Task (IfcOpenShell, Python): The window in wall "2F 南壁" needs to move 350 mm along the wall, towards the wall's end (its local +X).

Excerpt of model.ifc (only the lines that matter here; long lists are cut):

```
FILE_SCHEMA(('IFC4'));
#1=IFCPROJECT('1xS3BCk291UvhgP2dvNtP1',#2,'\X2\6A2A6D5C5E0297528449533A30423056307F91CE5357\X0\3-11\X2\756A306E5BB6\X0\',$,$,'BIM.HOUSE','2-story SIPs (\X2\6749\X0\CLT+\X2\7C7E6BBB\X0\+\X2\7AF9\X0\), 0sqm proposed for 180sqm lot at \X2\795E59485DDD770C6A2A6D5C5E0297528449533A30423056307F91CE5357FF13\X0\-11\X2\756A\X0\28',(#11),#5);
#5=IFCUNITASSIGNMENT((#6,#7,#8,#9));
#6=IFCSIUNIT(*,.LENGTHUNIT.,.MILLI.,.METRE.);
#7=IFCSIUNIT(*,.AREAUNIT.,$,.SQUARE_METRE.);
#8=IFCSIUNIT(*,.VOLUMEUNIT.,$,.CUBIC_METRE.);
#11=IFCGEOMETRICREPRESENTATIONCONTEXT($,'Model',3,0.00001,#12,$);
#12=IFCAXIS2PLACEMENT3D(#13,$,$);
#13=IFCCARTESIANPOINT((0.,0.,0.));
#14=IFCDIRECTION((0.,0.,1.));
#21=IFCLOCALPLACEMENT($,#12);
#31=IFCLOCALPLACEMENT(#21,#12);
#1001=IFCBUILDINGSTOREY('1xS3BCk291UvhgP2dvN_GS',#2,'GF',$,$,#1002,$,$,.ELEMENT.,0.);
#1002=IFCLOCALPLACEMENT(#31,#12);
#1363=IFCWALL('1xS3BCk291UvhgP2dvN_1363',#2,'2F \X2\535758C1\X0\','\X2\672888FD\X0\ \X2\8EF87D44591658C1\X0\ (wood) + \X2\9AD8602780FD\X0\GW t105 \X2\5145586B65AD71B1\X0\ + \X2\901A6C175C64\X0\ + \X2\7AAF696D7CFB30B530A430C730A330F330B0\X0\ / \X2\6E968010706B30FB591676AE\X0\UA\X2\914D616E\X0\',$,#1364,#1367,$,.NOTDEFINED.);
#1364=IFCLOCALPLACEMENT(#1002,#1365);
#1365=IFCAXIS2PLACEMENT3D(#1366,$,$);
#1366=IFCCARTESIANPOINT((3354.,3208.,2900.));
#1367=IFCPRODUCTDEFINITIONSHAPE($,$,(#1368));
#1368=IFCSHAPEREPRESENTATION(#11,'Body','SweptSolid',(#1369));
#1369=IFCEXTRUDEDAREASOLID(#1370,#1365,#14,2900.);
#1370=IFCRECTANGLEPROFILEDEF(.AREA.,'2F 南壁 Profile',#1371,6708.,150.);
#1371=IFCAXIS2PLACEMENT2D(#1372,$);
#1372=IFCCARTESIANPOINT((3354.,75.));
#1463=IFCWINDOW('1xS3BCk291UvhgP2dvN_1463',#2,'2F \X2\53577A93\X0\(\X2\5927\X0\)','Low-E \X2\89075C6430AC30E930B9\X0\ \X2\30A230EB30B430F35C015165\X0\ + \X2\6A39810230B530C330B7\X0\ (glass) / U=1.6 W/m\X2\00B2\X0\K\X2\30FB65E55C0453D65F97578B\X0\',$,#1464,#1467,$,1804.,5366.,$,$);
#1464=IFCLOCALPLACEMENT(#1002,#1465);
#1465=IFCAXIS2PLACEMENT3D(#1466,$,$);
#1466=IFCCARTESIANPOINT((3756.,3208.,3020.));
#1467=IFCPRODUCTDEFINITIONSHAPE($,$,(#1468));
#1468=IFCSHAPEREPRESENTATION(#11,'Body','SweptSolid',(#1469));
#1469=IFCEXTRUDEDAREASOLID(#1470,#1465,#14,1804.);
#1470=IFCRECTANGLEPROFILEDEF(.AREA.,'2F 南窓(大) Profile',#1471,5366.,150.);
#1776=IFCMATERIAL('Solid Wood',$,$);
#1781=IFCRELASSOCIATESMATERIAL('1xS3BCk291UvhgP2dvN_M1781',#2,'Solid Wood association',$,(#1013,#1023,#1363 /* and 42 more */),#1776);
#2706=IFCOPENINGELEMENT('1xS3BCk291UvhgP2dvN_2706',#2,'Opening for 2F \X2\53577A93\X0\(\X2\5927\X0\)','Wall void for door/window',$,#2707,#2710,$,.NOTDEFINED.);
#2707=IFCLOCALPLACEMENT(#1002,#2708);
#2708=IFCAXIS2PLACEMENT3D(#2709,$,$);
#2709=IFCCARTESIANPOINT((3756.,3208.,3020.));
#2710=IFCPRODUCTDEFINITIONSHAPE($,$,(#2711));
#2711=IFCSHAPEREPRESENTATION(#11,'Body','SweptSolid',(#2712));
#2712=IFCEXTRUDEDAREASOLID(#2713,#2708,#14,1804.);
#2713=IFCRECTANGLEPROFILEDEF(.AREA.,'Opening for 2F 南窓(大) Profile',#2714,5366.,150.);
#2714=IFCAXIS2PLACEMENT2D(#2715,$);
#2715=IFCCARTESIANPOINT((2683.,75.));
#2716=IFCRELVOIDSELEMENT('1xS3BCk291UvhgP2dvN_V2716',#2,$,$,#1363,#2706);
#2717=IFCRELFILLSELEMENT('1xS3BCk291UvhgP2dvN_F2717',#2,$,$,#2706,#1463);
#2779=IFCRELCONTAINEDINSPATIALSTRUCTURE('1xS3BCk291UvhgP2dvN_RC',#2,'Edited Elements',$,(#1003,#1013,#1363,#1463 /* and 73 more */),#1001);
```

```python
import ifcopenshell
import ifcopenshell.api.geometry
import ifcopenshell.util.placement

model = ifcopenshell.open("model.ifc")

window = model.by_guid("1xS3BCk291UvhgP2dvN_1463")
opening = window.FillsVoids[0].RelatingOpeningElement
wall = opening.VoidsElements[0].RelatingBuildingElement

wall_matrix = ifcopenshell.util.placement.get_local_placement(wall.ObjectPlacement)
shift = wall_matrix[:3, 0] * 350.0
before = ifcopenshell.util.placement.get_local_placement(window.ObjectPlacement)[:3, 3].copy()

# The window is not placed relative to its opening, so move both.
for product in (opening, window):
    matrix = ifcopenshell.util.placement.get_local_placement(product.ObjectPlacement)
    matrix[:3, 3] += shift
    ifcopenshell.api.geometry.edit_object_placement(model, product=product, matrix=matrix, is_si=False)

after = ifcopenshell.util.placement.get_local_placement(window.ObjectPlacement)[:3, 3]
print("window moved by", (after - before).round(3) + 0.0)

model.write("model_edited.ifc")
```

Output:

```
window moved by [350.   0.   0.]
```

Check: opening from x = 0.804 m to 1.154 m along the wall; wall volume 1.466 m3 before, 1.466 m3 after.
